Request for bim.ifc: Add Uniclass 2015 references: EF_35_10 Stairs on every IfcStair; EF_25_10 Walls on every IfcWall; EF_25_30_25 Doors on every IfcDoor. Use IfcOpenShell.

First a look at what the model holds.

```python
import ifcopenshell

model = ifcopenshell.open("bim.ifc")
print(model.schema)
print("classifications:", [c.Name for c in model.by_type("IfcClassification")])
for ifc_class in ("IfcDoor", "IfcRoof", "IfcStair", "IfcWall", "IfcWindow"):
    print(ifc_class, len(model.by_type(ifc_class)))
```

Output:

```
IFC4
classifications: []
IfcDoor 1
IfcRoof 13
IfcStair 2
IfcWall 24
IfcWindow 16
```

```python
import ifcopenshell
import ifcopenshell.api.classification

model = ifcopenshell.open("bim.ifc")

system = ifcopenshell.api.classification.add_classification(model, classification="Uniclass 2015")

codes = {
    "IfcStair": ("EF_35_10", "Stairs"),
    "IfcWall": ("EF_25_10", "Walls"),
    "IfcDoor": ("EF_25_30_25", "Doors"),
}
for ifc_class, (code, name) in codes.items():
    products = model.by_type(ifc_class)
    ifcopenshell.api.classification.add_reference(
        model, products=products, classification=system, identification=code, name=name
    )
    print(code, len(products))

model.write("bim_updated.ifc")
```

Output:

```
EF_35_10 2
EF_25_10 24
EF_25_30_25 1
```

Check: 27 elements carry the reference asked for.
